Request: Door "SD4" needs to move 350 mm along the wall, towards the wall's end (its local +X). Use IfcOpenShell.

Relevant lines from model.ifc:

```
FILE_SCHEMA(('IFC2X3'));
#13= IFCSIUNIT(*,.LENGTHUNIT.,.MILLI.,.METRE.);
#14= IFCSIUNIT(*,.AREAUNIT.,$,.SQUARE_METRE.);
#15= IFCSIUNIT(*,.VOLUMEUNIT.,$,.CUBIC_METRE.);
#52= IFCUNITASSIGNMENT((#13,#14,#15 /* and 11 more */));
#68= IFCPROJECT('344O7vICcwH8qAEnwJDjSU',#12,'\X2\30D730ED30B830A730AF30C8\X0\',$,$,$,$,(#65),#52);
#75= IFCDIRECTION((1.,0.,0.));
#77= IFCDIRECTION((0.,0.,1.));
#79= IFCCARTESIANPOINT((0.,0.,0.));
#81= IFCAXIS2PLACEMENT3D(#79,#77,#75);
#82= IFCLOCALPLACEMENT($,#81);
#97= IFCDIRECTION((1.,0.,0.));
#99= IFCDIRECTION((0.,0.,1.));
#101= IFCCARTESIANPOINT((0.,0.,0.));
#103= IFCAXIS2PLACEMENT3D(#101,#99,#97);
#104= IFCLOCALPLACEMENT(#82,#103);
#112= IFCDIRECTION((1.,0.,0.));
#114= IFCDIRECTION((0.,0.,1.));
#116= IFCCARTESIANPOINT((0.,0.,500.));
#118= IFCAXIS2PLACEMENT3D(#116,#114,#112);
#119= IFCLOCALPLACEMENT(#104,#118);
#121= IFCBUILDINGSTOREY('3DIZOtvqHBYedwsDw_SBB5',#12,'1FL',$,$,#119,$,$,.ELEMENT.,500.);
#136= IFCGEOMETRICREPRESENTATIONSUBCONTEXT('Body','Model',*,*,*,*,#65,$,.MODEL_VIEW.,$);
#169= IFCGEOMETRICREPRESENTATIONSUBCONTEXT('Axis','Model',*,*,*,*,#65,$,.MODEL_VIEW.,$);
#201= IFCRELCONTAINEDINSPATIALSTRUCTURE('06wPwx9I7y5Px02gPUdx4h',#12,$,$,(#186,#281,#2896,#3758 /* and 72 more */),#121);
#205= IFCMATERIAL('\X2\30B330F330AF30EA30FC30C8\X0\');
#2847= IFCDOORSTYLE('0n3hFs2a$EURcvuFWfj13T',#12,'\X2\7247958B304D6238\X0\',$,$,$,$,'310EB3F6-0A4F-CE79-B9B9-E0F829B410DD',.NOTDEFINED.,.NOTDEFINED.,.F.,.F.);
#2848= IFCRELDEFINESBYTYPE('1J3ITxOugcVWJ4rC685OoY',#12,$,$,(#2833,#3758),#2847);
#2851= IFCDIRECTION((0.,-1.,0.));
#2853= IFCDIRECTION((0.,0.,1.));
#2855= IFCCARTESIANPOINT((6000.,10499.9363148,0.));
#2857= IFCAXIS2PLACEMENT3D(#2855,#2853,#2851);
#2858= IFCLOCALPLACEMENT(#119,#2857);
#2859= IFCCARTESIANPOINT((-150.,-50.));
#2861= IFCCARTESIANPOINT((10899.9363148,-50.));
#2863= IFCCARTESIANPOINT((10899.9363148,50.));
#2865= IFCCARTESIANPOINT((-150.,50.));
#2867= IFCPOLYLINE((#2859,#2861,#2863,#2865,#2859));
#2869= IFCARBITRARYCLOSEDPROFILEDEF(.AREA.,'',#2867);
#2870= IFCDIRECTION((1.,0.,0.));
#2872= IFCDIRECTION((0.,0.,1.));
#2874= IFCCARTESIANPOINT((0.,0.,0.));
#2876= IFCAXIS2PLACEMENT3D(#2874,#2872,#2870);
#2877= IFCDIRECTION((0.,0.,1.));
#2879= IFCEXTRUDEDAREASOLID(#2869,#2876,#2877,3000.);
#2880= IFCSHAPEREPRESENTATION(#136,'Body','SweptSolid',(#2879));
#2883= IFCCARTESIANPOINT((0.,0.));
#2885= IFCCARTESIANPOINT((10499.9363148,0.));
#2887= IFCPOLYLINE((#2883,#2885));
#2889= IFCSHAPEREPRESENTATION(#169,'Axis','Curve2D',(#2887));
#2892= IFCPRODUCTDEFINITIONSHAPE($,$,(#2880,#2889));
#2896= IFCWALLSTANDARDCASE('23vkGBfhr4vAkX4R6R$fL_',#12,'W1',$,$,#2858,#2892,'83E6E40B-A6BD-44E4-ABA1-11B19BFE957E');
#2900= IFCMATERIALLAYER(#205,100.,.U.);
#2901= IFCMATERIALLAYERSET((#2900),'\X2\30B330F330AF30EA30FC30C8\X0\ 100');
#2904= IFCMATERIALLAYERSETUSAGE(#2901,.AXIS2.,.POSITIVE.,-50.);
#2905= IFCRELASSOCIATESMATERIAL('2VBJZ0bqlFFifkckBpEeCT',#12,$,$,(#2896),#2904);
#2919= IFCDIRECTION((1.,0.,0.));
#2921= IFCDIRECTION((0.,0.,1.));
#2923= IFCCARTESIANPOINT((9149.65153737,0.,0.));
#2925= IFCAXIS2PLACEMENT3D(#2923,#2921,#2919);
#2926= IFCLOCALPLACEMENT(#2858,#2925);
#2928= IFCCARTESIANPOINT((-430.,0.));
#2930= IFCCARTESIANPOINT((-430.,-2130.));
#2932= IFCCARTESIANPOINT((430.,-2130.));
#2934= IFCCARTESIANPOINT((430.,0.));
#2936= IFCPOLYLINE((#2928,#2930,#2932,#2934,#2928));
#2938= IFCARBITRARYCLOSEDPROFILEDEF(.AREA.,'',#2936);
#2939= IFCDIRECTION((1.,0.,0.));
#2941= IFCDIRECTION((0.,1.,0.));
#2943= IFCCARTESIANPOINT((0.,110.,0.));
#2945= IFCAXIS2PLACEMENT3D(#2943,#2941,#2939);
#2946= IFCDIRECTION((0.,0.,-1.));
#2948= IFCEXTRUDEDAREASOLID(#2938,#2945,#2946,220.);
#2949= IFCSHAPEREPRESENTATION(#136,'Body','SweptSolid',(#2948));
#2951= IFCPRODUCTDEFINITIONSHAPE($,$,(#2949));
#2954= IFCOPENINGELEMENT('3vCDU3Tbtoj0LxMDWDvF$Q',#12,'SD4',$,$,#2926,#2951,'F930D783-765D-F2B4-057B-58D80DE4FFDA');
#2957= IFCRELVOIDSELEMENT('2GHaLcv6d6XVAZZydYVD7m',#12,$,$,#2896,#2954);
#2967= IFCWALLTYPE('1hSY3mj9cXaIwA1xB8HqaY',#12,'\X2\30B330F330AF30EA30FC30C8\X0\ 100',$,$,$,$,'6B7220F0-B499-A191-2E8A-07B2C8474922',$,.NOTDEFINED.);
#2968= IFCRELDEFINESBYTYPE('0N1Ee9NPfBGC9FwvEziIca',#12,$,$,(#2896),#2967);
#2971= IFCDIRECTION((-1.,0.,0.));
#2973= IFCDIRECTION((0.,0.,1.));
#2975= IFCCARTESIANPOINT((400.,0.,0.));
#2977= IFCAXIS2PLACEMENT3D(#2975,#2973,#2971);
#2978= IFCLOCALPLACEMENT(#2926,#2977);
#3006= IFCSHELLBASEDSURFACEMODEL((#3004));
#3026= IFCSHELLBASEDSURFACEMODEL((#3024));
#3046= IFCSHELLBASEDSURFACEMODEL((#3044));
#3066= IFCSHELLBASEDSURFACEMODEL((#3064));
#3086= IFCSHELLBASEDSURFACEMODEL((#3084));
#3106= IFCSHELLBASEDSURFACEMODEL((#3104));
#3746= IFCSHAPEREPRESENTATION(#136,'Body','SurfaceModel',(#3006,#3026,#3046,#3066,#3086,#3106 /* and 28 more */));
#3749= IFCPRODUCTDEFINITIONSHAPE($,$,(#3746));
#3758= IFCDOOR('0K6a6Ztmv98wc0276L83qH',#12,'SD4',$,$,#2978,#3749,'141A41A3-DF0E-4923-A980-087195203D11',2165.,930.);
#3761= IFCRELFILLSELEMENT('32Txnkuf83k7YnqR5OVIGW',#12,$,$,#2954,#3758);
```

```python
import ifcopenshell
import ifcopenshell.api.geometry
import ifcopenshell.util.placement

model = ifcopenshell.open("model.ifc")

door = model.by_guid("0K6a6Ztmv98wc0276L83qH")
opening = door.FillsVoids[0].RelatingOpeningElement
wall = opening.VoidsElements[0].RelatingBuildingElement

wall_matrix = ifcopenshell.util.placement.get_local_placement(wall.ObjectPlacement)
shift = wall_matrix[:3, 0] * 350.0
before = ifcopenshell.util.placement.get_local_placement(door.ObjectPlacement)[:3, 3].copy()

# The door is placed relative to its opening, so it follows when the opening moves.
matrix = ifcopenshell.util.placement.get_local_placement(opening.ObjectPlacement)
matrix[:3, 3] += shift
ifcopenshell.api.geometry.edit_object_placement(
    model, product=opening, matrix=matrix, is_si=False, should_transform_children=True
)

after = ifcopenshell.util.placement.get_local_placement(door.ObjectPlacement)[:3, 3]
print("door moved by", (after - before).round(3) + 0.0)

model.write("model_v2.ifc")
```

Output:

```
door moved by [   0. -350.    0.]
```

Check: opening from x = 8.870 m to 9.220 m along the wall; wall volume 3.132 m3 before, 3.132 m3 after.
